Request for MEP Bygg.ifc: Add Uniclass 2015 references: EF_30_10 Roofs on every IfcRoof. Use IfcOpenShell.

First a look at what the model holds.

```python
import ifcopenshell

model = ifcopenshell.open("MEP Bygg.ifc")
print(model.schema)
print("classifications:", [c.Name for c in model.by_type("IfcClassification")])
for ifc_class in ("IfcDoor", "IfcRoof", "IfcStair", "IfcWall", "IfcWindow"):
    print(ifc_class, len(model.by_type(ifc_class)))
```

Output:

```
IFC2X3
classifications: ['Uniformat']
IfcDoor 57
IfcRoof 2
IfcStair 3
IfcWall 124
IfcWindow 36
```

```python
import ifcopenshell
import ifcopenshell.api.classification

model = ifcopenshell.open("MEP Bygg.ifc")

# IFC2X3 requires Source and Edition and has no link from the project to the system.
system = model.create_entity("IfcClassification", Source="NBS", Edition="2015", Name="Uniclass 2015")

codes = {
    "IfcRoof": ("EF_30_10", "Roofs"),
}
for ifc_class, (code, name) in codes.items():
    products = model.by_type(ifc_class)
    ifcopenshell.api.classification.add_reference(
        model, products=products, classification=system, identification=code, name=name
    )
    print(code, len(products))

model.write("MEP Bygg_rev.ifc")
```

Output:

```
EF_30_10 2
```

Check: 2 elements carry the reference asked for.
